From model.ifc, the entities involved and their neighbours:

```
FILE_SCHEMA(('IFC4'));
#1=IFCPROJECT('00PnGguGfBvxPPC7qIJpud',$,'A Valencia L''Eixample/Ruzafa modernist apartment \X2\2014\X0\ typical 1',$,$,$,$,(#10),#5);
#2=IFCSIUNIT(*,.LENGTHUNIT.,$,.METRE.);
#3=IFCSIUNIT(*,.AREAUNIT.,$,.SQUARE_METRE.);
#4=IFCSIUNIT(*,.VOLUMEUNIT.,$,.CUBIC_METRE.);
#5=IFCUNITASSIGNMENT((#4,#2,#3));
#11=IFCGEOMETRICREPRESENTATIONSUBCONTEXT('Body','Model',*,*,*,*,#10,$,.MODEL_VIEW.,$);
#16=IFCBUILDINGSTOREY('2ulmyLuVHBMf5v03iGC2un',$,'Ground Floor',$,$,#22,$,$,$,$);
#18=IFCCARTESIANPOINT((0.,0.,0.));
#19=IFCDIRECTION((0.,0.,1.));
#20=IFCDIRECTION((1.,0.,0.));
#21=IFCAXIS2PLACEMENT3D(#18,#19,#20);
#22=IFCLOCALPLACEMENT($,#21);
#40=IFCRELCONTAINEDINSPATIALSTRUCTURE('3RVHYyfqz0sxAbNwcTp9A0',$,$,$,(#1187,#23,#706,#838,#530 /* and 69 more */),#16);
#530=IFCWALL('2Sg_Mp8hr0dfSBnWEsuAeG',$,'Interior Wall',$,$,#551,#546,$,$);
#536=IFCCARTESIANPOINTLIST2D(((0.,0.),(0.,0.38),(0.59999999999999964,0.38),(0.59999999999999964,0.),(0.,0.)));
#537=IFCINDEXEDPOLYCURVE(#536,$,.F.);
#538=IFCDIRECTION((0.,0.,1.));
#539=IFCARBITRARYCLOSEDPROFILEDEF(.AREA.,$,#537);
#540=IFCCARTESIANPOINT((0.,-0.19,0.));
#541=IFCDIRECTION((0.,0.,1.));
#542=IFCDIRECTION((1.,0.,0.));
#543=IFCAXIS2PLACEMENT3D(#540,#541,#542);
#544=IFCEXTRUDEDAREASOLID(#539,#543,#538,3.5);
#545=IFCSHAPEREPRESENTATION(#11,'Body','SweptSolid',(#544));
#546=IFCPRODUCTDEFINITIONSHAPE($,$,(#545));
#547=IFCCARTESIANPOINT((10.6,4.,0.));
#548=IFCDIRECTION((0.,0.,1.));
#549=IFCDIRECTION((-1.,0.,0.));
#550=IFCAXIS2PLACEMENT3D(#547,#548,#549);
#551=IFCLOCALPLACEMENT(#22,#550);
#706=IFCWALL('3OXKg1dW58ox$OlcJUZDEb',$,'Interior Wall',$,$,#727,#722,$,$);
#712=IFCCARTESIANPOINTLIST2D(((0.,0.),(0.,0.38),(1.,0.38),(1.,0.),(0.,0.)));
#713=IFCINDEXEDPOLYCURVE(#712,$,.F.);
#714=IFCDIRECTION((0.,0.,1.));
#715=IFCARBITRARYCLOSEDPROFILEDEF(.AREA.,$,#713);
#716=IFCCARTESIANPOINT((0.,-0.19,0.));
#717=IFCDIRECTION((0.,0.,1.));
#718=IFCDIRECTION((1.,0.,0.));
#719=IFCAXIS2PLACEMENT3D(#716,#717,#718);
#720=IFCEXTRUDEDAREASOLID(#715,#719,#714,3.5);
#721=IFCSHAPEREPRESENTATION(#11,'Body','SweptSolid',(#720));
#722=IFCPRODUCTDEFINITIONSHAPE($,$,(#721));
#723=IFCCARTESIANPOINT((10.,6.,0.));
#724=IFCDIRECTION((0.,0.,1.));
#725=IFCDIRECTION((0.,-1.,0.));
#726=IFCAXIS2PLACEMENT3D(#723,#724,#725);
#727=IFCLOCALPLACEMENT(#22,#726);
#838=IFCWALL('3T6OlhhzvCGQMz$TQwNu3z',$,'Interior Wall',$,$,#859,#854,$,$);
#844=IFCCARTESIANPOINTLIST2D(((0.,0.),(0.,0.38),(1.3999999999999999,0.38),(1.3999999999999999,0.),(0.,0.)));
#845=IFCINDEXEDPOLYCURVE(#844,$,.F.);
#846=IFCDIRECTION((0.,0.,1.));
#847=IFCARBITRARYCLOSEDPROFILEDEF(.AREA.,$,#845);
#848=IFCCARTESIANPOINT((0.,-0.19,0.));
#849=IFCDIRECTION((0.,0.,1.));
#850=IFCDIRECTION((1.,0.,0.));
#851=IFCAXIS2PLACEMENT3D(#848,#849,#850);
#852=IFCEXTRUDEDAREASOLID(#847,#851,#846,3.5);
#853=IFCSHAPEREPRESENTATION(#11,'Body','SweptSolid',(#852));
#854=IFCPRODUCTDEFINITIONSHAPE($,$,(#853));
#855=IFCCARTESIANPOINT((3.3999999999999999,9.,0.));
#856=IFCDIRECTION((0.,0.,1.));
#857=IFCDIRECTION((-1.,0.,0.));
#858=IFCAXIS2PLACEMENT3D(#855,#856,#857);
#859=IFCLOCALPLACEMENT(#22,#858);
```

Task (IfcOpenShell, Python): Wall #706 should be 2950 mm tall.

```python
import ifcopenshell
import ifcopenshell.geom
import ifcopenshell.util.representation
import ifcopenshell.util.shape

model = ifcopenshell.open("model.ifc")
settings = ifcopenshell.geom.settings()


def volume(element):
    """Net volume in cubic metres, openings subtracted."""
    shape = ifcopenshell.geom.create_shape(settings, element)
    return ifcopenshell.util.shape.get_volume(shape.geometry)


wall = model.by_id(706)
before = volume(wall)

body = ifcopenshell.util.representation.get_representation(wall, "Model", "Body")
solid = body.Items[0]
old_height = solid.Depth
solid.Depth = 2.95
after = volume(wall)

print(f"height {old_height:g} -> {solid.Depth:g}, volume {before:.3f} -> {after:.3f} m3")

model.write("model_v2.ifc")
```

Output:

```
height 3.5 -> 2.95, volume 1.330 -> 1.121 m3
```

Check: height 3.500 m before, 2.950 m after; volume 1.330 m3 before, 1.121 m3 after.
